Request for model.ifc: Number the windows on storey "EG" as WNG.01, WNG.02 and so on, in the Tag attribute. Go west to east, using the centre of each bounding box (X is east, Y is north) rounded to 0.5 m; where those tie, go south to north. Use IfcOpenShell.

First a look at what the model holds.

```python
import ifcopenshell
import ifcopenshell.util.element
import ifcopenshell.util.placement

model = ifcopenshell.open("model.ifc")
print(model.schema)
storey = next(s for s in model.by_type("IfcBuildingStorey") if s.Name == "EG")
windows = [e for e in ifcopenshell.util.element.get_decomposition(storey) if e.is_a("IfcWindow")]
for e in sorted(windows, key=lambda e: e.id()):
    origin = ifcopenshell.util.placement.get_local_placement(e.ObjectPlacement)[:3, 3]
    print(e.id(), e.Tag, e.Name, origin.round(2) + 0.0, sep=" | ")
```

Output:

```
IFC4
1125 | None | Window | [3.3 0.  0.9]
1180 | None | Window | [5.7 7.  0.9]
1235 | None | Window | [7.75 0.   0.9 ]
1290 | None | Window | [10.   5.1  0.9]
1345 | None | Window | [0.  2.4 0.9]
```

```python
import ifcopenshell
import ifcopenshell.geom
import ifcopenshell.util.element
import ifcopenshell.util.shape

model = ifcopenshell.open("model.ifc")
settings = ifcopenshell.geom.settings()
settings.set("use-world-coords", True)


def centre(element):
    shape = ifcopenshell.geom.create_shape(settings, element)
    return ifcopenshell.util.shape.get_bbox_centroid(shape.geometry)


storey = next(s for s in model.by_type("IfcBuildingStorey") if s.Name == "EG")
windows = [e for e in ifcopenshell.util.element.get_decomposition(storey) if e.is_a("IfcWindow")]

# Insertion points can sit at a corner or the storey origin, so sort by the geometry (in metres).
centres = {e: centre(e) for e in windows}
windows.sort(key=lambda e: (round(centres[e][0] / 0.5), centres[e][1]))

for i, e in enumerate(windows, start=1):
    number = f"WNG.{i:02d}"
    e.Tag = number
    print(e.id(), number)

model.write("model_rev.ifc")
```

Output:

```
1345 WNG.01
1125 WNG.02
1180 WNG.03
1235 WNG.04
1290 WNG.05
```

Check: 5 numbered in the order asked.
